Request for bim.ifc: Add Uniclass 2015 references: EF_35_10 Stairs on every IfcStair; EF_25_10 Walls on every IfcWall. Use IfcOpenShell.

First a look at what the model holds.

```python
import ifcopenshell

model = ifcopenshell.open("bim.ifc")
print(model.schema)
print("classifications:", [c.Name for c in model.by_type("IfcClassification")])
for ifc_class in ("IfcDoor", "IfcRoof", "IfcStair", "IfcWall", "IfcWindow"):
    print(ifc_class, len(model.by_type(ifc_class)))
```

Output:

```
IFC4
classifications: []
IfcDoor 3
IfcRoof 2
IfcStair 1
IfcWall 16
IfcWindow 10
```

```python
import ifcopenshell
import ifcopenshell.api.classification

model = ifcopenshell.open("bim.ifc")

system = ifcopenshell.api.classification.add_classification(model, classification="Uniclass 2015")

codes = {
    "IfcStair": ("EF_35_10", "Stairs"),
    "IfcWall": ("EF_25_10", "Walls"),
}
for ifc_class, (code, name) in codes.items():
    products = model.by_type(ifc_class)
    ifcopenshell.api.classification.add_reference(
        model, products=products, classification=system, identification=code, name=name
    )
    print(code, len(products))

model.write("bim-out.ifc")
```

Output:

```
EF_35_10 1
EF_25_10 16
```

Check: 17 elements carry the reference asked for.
